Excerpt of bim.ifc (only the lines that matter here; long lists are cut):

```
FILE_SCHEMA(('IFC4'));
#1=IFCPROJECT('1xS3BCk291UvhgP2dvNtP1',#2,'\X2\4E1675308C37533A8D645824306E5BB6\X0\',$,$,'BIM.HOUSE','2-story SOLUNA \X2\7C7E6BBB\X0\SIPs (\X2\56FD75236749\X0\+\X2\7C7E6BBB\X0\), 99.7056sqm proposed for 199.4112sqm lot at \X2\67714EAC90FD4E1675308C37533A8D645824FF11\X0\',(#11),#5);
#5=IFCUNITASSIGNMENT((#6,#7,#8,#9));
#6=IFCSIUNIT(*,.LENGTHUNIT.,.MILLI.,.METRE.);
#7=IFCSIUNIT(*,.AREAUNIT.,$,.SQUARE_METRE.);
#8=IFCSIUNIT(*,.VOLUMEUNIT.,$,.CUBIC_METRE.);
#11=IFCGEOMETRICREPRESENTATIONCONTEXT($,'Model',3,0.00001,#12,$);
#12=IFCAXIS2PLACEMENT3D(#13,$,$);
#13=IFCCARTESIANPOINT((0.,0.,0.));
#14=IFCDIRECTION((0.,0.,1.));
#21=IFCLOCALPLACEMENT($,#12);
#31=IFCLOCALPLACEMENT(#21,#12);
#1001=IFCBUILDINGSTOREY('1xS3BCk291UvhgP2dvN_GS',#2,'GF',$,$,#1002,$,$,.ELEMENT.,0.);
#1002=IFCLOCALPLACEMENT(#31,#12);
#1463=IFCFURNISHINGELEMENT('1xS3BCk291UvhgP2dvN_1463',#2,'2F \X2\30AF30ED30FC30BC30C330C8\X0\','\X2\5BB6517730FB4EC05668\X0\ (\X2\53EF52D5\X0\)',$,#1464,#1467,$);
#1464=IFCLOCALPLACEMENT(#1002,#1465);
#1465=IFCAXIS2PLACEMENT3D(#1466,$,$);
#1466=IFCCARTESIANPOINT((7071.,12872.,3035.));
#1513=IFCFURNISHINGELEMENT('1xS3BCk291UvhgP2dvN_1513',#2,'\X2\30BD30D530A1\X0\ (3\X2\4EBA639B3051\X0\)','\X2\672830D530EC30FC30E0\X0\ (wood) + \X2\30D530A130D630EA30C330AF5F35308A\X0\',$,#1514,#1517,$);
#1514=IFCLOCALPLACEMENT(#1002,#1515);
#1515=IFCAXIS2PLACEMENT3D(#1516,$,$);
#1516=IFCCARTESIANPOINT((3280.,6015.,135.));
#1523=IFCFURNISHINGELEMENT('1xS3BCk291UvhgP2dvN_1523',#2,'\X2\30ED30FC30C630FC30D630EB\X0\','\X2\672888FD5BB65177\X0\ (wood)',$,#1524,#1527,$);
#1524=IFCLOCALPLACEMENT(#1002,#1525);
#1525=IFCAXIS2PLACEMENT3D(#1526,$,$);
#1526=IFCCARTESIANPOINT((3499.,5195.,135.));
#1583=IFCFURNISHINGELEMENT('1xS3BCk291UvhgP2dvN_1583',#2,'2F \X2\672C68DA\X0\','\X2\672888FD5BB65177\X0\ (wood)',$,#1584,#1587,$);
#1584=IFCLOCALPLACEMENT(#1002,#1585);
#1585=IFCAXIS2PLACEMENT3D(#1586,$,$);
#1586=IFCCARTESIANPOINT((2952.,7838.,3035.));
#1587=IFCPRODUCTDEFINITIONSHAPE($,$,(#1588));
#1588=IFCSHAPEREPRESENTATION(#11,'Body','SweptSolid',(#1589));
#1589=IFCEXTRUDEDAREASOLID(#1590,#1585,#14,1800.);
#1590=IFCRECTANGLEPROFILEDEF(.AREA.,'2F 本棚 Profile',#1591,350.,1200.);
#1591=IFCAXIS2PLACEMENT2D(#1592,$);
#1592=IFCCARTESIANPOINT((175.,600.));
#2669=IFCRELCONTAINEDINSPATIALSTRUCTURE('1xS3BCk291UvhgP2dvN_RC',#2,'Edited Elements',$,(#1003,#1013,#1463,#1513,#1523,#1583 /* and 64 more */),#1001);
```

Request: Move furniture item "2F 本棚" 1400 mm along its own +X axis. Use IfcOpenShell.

```python
import ifcopenshell
import ifcopenshell.api.geometry
import ifcopenshell.util.placement
import ifcopenshell.util.unit

model = ifcopenshell.open("bim.ifc")
unit_scale = ifcopenshell.util.unit.calculate_unit_scale(model)

item = model.by_guid("1xS3BCk291UvhgP2dvN_1583")
matrix = ifcopenshell.util.placement.get_local_placement(item.ObjectPlacement)
matrix[:3, 3] += matrix[:3, 0] * 1.4 / unit_scale
ifcopenshell.api.geometry.edit_object_placement(model, product=item, matrix=matrix, is_si=False)

print(ifcopenshell.util.placement.get_local_placement(item.ObjectPlacement).round(3) + 0.0)

model.write("bim_v2.ifc")
```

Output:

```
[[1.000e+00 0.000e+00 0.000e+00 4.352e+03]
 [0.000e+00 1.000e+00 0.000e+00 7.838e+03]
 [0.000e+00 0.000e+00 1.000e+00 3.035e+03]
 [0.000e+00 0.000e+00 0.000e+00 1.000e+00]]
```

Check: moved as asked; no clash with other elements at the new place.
